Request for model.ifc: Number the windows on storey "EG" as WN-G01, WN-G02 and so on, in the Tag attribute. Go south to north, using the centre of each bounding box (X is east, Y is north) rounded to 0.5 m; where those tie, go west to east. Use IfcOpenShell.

First a look at what the model holds.

```python
import ifcopenshell
import ifcopenshell.util.element
import ifcopenshell.util.placement

model = ifcopenshell.open("model.ifc")
print(model.schema)
storey = next(s for s in model.by_type("IfcBuildingStorey") if s.Name == "EG")
windows = [e for e in ifcopenshell.util.element.get_decomposition(storey) if e.is_a("IfcWindow")]
for e in sorted(windows, key=lambda e: e.id()):
    origin = ifcopenshell.util.placement.get_local_placement(e.ObjectPlacement)[:3, 3]
    print(e.id(), e.Tag, e.Name, origin.round(2) + 0.0, sep=" | ")
```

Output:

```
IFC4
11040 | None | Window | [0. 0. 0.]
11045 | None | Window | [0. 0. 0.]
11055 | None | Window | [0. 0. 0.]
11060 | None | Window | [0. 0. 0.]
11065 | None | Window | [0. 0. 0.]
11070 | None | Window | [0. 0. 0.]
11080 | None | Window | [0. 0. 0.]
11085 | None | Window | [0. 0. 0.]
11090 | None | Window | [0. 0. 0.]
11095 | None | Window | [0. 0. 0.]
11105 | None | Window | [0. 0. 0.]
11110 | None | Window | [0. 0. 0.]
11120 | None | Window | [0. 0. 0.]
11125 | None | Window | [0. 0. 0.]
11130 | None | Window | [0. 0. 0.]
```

```python
import ifcopenshell
import ifcopenshell.geom
import ifcopenshell.util.element
import ifcopenshell.util.shape

model = ifcopenshell.open("model.ifc")
settings = ifcopenshell.geom.settings()
settings.set("use-world-coords", True)


def centre(element):
    shape = ifcopenshell.geom.create_shape(settings, element)
    return ifcopenshell.util.shape.get_bbox_centroid(shape.geometry)


storey = next(s for s in model.by_type("IfcBuildingStorey") if s.Name == "EG")
windows = [e for e in ifcopenshell.util.element.get_decomposition(storey) if e.is_a("IfcWindow")]

# Insertion points can sit at a corner or the storey origin, so sort by the geometry (in metres).
centres = {e: centre(e) for e in windows}
windows.sort(key=lambda e: (round(centres[e][1] / 0.5), centres[e][0]))

for i, e in enumerate(windows, start=1):
    number = f"WN-G{i:02d}"
    e.Tag = number
    print(e.id(), number)

model.write("model_updated.ifc")
```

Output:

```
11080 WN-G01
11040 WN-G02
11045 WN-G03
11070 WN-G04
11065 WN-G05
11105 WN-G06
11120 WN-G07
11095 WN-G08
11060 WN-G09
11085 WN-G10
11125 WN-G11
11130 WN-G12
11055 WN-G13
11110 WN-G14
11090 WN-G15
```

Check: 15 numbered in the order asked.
